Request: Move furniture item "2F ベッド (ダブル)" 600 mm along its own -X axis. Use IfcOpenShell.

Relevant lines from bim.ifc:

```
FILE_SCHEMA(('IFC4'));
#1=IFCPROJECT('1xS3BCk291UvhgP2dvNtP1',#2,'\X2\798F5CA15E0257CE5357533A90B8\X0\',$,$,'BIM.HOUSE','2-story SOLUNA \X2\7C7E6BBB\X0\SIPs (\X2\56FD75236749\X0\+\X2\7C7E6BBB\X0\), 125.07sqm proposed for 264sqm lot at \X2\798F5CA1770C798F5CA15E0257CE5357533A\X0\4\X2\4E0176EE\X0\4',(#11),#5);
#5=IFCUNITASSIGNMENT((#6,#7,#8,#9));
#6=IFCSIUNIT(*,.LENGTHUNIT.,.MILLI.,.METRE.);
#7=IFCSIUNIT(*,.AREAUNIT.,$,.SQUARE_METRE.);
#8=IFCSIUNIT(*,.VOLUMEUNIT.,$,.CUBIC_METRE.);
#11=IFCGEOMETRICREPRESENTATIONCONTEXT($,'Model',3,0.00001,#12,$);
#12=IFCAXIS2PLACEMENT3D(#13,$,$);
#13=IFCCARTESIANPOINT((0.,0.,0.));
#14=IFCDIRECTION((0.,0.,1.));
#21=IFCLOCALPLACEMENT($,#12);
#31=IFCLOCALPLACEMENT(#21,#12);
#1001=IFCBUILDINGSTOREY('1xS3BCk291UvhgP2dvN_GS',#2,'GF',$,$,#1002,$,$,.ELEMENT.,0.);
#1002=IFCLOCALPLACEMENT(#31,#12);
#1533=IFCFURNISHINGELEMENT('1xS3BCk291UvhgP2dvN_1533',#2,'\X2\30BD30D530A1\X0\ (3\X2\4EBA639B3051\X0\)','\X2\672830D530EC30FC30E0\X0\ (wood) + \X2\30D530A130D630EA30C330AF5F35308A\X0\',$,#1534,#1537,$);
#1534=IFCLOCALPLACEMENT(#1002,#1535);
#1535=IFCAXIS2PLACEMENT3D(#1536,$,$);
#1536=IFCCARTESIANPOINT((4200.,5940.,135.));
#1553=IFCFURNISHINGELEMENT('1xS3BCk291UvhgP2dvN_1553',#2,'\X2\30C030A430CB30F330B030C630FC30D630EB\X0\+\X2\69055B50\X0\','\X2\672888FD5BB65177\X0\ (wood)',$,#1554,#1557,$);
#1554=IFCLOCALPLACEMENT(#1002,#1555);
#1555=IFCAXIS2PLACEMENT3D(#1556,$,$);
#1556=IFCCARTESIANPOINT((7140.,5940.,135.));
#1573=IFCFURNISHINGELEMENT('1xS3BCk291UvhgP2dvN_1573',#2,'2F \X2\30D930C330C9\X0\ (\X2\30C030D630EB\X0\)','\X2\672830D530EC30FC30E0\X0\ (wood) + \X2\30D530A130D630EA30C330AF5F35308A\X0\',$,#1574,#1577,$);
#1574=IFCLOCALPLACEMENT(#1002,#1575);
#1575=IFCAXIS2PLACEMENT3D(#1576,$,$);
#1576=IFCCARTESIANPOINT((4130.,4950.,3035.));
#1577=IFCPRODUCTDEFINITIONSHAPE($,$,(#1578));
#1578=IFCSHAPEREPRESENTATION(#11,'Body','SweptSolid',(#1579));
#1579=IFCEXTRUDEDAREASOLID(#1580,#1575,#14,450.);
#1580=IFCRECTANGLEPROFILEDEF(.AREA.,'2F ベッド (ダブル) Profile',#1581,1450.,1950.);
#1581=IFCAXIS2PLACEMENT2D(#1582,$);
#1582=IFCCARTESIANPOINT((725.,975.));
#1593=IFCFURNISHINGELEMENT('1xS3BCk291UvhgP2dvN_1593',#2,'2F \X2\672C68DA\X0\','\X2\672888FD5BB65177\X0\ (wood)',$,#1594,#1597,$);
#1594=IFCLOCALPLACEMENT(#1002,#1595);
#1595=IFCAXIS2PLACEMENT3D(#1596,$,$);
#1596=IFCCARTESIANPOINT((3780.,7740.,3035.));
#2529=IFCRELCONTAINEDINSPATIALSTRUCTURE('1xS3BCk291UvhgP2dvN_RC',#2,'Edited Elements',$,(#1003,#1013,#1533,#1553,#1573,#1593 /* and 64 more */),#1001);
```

```python
import ifcopenshell
import ifcopenshell.api.geometry
import ifcopenshell.util.placement
import ifcopenshell.util.unit

model = ifcopenshell.open("bim.ifc")
unit_scale = ifcopenshell.util.unit.calculate_unit_scale(model)

item = model.by_guid("1xS3BCk291UvhgP2dvN_1573")
matrix = ifcopenshell.util.placement.get_local_placement(item.ObjectPlacement)
matrix[:3, 3] -= matrix[:3, 0] * 0.6 / unit_scale
ifcopenshell.api.geometry.edit_object_placement(model, product=item, matrix=matrix, is_si=False)

print(ifcopenshell.util.placement.get_local_placement(item.ObjectPlacement).round(3) + 0.0)

model.write("bim_rev.ifc")
```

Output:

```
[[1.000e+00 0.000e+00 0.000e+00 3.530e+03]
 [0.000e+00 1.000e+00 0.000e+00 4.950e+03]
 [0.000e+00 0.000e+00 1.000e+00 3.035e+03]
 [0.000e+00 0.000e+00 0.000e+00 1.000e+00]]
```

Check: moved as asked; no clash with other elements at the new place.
